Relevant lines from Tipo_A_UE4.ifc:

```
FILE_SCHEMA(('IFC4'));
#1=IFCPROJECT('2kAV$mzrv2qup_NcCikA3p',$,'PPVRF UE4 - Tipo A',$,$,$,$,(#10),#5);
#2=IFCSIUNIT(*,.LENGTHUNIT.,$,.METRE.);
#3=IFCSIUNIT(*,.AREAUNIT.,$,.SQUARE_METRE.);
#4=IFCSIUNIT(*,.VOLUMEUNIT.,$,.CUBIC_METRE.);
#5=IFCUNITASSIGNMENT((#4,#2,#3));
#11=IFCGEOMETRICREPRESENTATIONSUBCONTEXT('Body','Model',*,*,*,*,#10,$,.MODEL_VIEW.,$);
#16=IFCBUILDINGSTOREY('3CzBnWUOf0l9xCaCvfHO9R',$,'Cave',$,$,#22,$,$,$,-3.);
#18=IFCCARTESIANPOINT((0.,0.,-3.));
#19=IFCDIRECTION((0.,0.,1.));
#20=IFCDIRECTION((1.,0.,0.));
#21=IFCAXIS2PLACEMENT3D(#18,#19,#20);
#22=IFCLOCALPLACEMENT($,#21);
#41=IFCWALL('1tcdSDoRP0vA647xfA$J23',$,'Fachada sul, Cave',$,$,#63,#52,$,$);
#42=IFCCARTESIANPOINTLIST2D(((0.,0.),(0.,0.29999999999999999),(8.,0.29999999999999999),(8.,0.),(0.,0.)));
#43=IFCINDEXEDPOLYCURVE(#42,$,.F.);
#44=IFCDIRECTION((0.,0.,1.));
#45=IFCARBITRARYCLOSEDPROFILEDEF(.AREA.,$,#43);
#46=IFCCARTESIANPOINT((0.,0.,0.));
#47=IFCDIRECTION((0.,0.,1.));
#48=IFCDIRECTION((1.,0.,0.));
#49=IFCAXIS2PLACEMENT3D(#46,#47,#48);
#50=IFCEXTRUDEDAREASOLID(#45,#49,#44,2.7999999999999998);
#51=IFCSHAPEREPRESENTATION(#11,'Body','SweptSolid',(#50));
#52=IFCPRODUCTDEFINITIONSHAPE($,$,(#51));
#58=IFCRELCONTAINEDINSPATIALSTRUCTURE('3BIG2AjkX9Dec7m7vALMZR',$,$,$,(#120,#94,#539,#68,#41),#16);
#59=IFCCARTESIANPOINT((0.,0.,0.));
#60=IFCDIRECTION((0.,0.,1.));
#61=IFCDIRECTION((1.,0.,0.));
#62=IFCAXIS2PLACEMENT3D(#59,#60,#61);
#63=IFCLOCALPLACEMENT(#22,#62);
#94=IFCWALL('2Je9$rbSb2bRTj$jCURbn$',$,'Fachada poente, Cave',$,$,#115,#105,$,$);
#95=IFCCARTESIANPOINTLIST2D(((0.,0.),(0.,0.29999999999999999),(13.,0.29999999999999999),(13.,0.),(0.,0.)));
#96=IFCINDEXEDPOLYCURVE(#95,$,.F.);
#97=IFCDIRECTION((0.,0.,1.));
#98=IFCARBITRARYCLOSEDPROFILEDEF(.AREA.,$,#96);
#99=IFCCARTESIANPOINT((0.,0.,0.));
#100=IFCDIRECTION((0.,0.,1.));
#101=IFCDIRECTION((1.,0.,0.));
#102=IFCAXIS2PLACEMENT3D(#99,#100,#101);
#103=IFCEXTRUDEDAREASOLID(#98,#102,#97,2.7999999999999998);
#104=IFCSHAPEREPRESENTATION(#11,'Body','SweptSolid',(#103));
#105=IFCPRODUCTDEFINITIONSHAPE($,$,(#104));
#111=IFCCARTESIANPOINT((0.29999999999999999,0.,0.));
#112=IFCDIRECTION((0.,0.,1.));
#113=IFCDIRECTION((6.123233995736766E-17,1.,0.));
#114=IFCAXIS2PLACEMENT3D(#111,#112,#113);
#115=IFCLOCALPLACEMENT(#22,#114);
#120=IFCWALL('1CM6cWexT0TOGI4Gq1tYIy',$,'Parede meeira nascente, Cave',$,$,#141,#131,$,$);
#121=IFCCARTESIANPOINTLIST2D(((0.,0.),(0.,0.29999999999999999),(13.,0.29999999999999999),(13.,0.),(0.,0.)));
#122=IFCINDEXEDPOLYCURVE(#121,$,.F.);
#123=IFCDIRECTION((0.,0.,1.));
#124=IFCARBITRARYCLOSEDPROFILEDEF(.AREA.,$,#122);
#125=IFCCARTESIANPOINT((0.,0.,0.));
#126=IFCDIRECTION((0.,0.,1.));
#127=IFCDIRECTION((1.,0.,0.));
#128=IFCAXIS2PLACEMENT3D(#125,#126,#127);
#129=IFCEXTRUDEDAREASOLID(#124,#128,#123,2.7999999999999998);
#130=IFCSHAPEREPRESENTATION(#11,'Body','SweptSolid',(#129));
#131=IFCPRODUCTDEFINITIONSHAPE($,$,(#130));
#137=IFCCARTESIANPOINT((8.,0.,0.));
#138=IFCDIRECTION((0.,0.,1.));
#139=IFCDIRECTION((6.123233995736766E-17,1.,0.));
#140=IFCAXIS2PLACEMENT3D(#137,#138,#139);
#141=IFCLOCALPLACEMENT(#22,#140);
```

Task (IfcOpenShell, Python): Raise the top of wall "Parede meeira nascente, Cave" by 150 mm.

```python
import ifcopenshell
import ifcopenshell.geom
import ifcopenshell.util.representation
import ifcopenshell.util.shape

model = ifcopenshell.open("Tipo_A_UE4.ifc")
settings = ifcopenshell.geom.settings()


def volume(element):
    """Net volume in cubic metres, openings subtracted."""
    shape = ifcopenshell.geom.create_shape(settings, element)
    return ifcopenshell.util.shape.get_volume(shape.geometry)


wall = model.by_id(120)
before = volume(wall)

body = ifcopenshell.util.representation.get_representation(wall, "Model", "Body")
solid = body.Items[0]
old_height = solid.Depth
solid.Depth += 0.15
after = volume(wall)

print(f"height {old_height:g} -> {solid.Depth:g}, volume {before:.3f} -> {after:.3f} m3")

model.write("Tipo_A_UE4_edited.ifc")
```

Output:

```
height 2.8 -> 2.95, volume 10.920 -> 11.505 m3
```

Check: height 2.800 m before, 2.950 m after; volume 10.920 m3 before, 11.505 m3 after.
